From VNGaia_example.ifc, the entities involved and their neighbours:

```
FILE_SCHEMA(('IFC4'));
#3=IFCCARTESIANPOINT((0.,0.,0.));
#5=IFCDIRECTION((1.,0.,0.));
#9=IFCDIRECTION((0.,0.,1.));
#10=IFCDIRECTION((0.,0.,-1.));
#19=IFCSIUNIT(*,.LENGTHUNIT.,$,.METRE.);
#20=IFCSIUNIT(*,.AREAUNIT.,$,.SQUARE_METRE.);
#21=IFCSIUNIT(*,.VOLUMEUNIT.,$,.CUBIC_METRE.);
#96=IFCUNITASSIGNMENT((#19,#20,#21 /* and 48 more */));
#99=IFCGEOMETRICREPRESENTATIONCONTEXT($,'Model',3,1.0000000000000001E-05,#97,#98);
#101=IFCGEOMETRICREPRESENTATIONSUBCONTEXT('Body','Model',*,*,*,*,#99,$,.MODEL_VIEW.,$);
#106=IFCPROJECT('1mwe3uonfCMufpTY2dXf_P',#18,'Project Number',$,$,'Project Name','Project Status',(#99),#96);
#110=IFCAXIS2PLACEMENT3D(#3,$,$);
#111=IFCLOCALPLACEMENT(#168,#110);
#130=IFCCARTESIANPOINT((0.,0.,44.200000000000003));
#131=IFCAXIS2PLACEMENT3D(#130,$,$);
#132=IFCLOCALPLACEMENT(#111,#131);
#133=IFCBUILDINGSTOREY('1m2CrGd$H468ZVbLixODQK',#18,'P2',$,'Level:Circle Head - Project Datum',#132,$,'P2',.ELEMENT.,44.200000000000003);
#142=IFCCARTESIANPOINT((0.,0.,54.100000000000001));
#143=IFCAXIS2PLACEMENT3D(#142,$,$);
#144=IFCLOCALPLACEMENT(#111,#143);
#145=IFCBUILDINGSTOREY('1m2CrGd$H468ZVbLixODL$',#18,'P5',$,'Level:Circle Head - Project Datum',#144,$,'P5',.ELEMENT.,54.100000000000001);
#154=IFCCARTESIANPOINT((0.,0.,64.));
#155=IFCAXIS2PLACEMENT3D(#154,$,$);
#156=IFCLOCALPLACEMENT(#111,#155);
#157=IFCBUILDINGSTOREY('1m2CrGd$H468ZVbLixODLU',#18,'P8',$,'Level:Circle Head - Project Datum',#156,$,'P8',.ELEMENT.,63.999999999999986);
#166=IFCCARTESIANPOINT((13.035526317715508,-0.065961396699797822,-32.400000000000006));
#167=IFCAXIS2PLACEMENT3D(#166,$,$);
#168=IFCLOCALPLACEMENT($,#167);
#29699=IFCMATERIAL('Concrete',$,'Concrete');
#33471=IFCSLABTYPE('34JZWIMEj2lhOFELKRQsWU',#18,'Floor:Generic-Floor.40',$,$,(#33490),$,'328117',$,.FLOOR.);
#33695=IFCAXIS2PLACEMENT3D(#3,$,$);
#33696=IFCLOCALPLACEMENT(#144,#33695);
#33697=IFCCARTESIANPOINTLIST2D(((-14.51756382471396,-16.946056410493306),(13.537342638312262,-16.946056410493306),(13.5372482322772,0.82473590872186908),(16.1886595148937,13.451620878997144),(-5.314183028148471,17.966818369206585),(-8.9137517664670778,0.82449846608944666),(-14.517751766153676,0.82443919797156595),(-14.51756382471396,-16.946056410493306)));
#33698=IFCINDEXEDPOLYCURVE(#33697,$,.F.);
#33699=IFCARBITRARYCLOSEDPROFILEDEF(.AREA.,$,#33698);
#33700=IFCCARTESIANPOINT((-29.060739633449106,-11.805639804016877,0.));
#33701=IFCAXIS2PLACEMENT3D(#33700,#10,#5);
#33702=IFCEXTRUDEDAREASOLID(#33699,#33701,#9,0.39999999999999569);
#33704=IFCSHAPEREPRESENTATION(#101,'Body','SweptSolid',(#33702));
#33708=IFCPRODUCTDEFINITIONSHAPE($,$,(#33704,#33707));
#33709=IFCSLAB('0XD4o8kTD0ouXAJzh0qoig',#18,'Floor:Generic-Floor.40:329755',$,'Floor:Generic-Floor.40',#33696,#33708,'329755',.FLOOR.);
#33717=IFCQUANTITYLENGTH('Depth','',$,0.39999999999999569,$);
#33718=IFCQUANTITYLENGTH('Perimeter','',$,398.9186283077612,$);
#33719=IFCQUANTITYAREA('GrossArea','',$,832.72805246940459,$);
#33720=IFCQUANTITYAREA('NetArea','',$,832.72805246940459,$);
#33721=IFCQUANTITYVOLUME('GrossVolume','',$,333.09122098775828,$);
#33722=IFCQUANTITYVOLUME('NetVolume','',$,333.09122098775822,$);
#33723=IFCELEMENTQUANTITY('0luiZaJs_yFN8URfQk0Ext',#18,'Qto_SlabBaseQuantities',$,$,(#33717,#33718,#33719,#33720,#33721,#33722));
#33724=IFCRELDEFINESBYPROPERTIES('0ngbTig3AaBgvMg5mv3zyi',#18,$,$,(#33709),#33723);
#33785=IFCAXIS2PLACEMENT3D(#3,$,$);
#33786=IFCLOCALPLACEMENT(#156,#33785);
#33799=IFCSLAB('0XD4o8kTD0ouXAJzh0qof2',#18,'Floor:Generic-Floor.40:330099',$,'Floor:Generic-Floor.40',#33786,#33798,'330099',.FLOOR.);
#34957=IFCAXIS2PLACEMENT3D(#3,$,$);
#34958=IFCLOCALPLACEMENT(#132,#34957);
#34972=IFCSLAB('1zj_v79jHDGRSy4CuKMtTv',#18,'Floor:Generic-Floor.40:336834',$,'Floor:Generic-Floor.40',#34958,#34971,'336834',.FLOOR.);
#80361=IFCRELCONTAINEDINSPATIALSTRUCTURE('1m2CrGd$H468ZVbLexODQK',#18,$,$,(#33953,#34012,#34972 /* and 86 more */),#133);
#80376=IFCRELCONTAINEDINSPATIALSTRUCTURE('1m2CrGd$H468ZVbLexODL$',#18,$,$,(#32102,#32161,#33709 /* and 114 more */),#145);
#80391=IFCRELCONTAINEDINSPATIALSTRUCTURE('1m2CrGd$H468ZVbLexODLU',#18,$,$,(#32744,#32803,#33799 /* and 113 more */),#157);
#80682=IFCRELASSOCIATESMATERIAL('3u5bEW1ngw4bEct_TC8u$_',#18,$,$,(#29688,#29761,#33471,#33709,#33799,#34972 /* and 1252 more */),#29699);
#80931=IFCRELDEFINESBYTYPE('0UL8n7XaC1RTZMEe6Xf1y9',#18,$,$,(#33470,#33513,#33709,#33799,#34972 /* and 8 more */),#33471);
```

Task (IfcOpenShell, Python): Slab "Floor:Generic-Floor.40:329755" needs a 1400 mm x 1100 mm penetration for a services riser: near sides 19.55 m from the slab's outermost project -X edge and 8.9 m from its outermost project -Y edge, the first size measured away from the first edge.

```python
import numpy as np
import ifcopenshell
import ifcopenshell.api.feature
import ifcopenshell.api.geometry
import ifcopenshell.api.pset
import ifcopenshell.api.root
import ifcopenshell.geom
import ifcopenshell.util.element
import ifcopenshell.util.placement
import ifcopenshell.util.representation
import ifcopenshell.util.shape
import ifcopenshell.util.unit

model = ifcopenshell.open("VNGaia_example.ifc")
unit_scale = ifcopenshell.util.unit.calculate_unit_scale(model)
area_scale = ifcopenshell.util.unit.calculate_unit_scale(model, "AREAUNIT")
volume_scale = ifcopenshell.util.unit.calculate_unit_scale(model, "VOLUMEUNIT")
settings = ifcopenshell.geom.settings()


def volume(element):
    """Net volume in cubic metres, openings subtracted."""
    shape = ifcopenshell.geom.create_shape(settings, element)
    return ifcopenshell.util.shape.get_volume(shape.geometry)


slab = model.by_id(33709)
before = volume(slab)

# Extent in the slab's own axes, in metres. The edges named are its -X and -Y sides.
slab_shape = ifcopenshell.geom.create_shape(settings, slab)
vertices = ifcopenshell.util.shape.get_vertices(slab_shape.geometry)
x_min, y_min, bottom = vertices.min(axis=0)
top = vertices[:, 2].max()

opening = ifcopenshell.api.root.create_entity(model, ifc_class="IfcOpeningElement", name="Services riser opening", predefined_type="OPENING")
context = ifcopenshell.util.representation.get_context(model, "Model", "Body", "MODEL_VIEW")
width, depth = 1.4, 1.1
outline = [(0.0, 0.0), (width, 0.0), (width, depth), (0.0, depth), (0.0, 0.0)]
# Overshoot both faces by 50 mm so the cut is clean.
shape = ifcopenshell.api.geometry.add_slab_representation(
    model, context=context, depth=top - bottom + 0.1, polyline=outline
)
ifcopenshell.api.geometry.assign_representation(model, product=opening, representation=shape)

matrix = ifcopenshell.util.placement.get_local_placement(slab.ObjectPlacement)
matrix[:, 3] = matrix @ np.append(np.array([x_min + 19.55, y_min + 8.9, bottom - 0.05]) / unit_scale, 1.0)
ifcopenshell.api.geometry.edit_object_placement(model, product=opening, matrix=matrix, is_si=False)
ifcopenshell.api.feature.add_feature(model, feature=opening, element=slab)

after = volume(slab)

# Update the slab's stored quantities.
qto = model.by_id(ifcopenshell.util.element.get_pset(slab, "Qto_SlabBaseQuantities", should_inherit=False)["id"])
ifcopenshell.api.pset.edit_qto(model, qto=qto, properties={
    "NetArea": after / (top - bottom) / area_scale,
    "NetVolume": after / volume_scale,
})

print(f"slab volume {before:.3f} -> {after:.3f} m3")

model.write("VNGaia_example_v2.ifc")
```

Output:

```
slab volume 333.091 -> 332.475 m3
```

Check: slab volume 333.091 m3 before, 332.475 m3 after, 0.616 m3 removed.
